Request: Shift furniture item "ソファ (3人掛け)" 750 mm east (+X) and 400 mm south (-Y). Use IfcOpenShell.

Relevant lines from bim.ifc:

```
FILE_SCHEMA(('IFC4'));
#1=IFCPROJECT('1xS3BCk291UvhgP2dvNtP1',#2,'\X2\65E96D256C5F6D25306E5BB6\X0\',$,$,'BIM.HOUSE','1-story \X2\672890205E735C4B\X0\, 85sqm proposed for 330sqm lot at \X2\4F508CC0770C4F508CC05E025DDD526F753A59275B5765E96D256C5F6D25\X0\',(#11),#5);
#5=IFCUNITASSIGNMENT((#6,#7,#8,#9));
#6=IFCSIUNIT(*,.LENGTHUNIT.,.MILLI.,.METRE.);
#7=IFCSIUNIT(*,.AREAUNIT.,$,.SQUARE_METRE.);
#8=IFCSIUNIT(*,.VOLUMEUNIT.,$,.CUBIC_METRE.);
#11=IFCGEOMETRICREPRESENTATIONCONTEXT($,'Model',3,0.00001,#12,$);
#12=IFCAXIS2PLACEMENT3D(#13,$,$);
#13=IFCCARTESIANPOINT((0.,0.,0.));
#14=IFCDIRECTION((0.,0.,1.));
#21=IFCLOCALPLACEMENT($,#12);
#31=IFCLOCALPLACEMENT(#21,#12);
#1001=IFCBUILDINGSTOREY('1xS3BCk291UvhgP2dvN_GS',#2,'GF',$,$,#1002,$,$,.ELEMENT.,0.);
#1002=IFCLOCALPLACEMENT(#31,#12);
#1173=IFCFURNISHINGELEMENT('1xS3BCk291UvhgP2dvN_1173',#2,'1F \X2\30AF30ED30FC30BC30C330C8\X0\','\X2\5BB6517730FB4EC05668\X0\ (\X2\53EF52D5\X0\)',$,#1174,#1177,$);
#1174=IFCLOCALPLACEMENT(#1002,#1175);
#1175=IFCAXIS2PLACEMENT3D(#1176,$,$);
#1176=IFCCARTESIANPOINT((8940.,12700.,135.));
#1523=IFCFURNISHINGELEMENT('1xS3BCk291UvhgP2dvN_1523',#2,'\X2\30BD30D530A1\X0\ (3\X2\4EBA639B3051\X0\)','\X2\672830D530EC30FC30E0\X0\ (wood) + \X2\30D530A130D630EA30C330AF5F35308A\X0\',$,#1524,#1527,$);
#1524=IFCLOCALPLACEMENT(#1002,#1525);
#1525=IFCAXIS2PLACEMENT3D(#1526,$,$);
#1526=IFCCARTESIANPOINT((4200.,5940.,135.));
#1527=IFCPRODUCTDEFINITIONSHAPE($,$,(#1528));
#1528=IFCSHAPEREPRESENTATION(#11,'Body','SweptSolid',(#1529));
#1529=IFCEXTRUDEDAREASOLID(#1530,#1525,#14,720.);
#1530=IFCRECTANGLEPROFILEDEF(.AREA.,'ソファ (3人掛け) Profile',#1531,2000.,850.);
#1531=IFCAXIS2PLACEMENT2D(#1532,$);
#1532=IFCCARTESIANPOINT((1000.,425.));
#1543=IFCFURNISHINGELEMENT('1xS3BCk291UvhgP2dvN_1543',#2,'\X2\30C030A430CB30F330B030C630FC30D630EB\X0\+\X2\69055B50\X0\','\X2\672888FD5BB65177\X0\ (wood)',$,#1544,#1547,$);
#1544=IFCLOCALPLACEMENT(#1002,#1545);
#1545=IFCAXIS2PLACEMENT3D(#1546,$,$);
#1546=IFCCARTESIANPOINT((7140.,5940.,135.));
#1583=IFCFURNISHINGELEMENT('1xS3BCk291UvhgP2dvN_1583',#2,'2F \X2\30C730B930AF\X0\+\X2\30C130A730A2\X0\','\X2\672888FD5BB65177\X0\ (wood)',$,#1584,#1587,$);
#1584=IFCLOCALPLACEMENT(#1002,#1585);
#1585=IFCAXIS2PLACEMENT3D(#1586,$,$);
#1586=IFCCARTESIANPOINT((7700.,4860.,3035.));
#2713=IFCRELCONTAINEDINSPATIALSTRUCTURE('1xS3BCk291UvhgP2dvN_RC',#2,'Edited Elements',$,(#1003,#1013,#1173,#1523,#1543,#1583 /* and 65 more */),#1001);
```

```python
import ifcopenshell
import ifcopenshell.api.geometry
import ifcopenshell.util.placement

model = ifcopenshell.open("bim.ifc")

item = model.by_id(1523)
matrix = ifcopenshell.util.placement.get_local_placement(item.ObjectPlacement)
matrix[0, 3] += 750.0
matrix[1, 3] -= 400.0
ifcopenshell.api.geometry.edit_object_placement(model, product=item, matrix=matrix, is_si=False)

print(ifcopenshell.util.placement.get_local_placement(item.ObjectPlacement).round(3) + 0.0)

model.write("bim_edited.ifc")
```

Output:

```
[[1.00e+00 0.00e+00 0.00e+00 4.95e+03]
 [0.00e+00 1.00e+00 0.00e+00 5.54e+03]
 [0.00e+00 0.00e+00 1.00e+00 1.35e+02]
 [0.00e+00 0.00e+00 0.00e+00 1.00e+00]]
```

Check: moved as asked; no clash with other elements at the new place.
